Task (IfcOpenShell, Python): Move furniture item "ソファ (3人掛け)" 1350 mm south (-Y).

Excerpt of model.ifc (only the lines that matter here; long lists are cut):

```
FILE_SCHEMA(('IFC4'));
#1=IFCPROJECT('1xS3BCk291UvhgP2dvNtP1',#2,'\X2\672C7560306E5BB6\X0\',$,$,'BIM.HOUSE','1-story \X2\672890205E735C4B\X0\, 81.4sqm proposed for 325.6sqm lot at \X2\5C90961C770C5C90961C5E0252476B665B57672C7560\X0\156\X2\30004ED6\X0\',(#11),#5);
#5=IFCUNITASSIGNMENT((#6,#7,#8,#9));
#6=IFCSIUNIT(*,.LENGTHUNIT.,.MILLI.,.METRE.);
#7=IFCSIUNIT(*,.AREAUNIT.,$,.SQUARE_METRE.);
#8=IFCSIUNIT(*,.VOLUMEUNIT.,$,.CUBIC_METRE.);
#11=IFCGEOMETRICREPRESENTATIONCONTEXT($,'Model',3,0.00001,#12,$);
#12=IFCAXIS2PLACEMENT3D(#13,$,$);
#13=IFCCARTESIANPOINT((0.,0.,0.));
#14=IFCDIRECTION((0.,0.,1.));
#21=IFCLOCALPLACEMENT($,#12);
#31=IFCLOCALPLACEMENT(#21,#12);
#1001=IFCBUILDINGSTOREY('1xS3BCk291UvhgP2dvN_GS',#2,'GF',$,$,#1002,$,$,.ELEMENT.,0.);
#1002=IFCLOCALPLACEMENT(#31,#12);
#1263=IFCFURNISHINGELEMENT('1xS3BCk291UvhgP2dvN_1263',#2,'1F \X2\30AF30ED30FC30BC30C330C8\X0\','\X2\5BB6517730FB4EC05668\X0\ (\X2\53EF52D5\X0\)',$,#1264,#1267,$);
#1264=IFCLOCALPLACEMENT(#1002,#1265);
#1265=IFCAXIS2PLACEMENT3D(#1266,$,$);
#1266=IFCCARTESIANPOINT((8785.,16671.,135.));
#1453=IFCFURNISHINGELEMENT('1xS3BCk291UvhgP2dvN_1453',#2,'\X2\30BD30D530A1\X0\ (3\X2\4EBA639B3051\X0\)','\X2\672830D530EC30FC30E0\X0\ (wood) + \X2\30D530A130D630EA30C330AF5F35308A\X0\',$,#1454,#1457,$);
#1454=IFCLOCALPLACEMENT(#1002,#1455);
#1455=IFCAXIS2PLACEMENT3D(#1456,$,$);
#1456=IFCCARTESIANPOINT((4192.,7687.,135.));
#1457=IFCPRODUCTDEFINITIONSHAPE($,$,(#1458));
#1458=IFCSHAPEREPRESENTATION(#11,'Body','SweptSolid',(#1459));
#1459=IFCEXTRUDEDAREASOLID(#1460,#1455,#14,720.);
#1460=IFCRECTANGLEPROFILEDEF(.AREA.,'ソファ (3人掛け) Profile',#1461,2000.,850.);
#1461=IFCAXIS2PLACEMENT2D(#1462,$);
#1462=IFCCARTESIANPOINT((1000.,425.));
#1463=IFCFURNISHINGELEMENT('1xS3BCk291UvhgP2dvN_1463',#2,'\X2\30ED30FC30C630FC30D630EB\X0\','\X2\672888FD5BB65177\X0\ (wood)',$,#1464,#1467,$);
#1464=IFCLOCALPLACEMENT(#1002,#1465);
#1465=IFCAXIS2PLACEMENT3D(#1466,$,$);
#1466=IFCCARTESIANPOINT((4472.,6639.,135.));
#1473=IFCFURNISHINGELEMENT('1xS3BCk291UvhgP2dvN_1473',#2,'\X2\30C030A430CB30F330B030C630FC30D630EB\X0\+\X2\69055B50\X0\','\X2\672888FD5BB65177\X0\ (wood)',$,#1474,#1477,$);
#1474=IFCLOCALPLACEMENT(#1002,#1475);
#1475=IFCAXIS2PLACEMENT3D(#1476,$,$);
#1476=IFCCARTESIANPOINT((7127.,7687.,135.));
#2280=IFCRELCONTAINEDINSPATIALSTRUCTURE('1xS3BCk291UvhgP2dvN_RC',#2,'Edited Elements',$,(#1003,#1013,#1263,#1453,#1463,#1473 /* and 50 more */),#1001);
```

```python
import ifcopenshell
import ifcopenshell.api.geometry
import ifcopenshell.util.placement
import ifcopenshell.util.unit

model = ifcopenshell.open("model.ifc")
unit_scale = ifcopenshell.util.unit.calculate_unit_scale(model)

item = model.by_id(1453)
matrix = ifcopenshell.util.placement.get_local_placement(item.ObjectPlacement)
matrix[1, 3] -= 1.35 / unit_scale
ifcopenshell.api.geometry.edit_object_placement(model, product=item, matrix=matrix, is_si=False)

print(ifcopenshell.util.placement.get_local_placement(item.ObjectPlacement).round(3) + 0.0)

model.write("model-out.ifc")
```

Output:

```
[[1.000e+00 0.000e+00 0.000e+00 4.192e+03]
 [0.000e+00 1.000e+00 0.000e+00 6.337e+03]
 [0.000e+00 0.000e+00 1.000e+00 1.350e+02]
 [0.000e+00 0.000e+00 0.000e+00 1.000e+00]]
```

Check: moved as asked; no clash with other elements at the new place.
